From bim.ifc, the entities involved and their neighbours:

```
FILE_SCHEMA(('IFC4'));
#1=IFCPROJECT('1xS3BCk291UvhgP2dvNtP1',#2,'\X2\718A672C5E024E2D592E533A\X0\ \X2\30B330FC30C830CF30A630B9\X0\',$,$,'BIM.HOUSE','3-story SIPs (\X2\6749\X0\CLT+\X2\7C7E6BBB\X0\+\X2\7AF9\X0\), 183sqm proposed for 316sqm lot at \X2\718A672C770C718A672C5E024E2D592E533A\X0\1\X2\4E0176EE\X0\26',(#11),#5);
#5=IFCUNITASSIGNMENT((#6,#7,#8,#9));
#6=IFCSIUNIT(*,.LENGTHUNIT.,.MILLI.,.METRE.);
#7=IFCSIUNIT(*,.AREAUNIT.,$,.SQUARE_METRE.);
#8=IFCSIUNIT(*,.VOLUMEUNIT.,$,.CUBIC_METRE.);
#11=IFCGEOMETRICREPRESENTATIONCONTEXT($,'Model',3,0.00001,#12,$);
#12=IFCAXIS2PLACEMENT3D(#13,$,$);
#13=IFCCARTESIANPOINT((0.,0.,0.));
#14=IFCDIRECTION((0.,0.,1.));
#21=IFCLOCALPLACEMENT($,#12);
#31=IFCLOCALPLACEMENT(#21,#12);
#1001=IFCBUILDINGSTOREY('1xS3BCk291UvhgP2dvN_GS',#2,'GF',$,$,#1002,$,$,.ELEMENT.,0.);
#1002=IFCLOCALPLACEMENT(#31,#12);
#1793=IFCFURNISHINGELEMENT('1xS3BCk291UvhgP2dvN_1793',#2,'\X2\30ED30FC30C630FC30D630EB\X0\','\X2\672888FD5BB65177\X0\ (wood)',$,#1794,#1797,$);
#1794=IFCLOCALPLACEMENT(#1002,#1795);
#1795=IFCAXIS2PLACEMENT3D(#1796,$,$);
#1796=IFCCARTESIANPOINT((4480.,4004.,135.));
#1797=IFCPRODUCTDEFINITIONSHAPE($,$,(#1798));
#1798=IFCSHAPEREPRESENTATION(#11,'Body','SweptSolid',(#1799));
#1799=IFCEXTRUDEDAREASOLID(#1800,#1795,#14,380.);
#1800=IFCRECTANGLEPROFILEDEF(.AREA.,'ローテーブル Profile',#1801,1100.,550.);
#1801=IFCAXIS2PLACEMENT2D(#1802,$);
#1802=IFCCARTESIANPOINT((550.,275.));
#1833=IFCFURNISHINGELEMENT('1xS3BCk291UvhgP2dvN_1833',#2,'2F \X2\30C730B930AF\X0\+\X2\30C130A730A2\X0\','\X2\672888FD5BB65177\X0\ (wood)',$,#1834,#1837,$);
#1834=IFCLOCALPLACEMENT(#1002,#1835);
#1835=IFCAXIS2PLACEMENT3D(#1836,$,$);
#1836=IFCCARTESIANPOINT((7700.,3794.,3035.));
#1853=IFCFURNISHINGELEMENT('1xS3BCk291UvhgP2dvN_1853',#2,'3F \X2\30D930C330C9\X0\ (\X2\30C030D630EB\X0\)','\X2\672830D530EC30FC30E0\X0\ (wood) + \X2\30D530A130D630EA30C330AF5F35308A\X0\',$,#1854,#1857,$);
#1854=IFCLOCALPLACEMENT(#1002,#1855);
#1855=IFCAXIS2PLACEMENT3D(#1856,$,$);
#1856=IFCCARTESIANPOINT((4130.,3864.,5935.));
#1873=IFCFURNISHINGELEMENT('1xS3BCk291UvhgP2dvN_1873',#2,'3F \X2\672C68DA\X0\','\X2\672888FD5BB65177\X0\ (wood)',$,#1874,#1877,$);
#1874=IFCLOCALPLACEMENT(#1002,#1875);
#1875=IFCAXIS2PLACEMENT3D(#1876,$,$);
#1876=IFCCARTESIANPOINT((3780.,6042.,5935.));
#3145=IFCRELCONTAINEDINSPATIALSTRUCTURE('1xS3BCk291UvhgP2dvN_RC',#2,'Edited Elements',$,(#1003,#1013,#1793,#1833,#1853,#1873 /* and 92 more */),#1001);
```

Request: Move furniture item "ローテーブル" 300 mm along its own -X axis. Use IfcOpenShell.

```python
import ifcopenshell
import ifcopenshell.api.geometry
import ifcopenshell.util.placement
import ifcopenshell.util.unit

model = ifcopenshell.open("bim.ifc")
unit_scale = ifcopenshell.util.unit.calculate_unit_scale(model)

item = model.by_id(1793)
matrix = ifcopenshell.util.placement.get_local_placement(item.ObjectPlacement)
matrix[:3, 3] -= matrix[:3, 0] * 0.3 / unit_scale
ifcopenshell.api.geometry.edit_object_placement(model, product=item, matrix=matrix, is_si=False)

print(ifcopenshell.util.placement.get_local_placement(item.ObjectPlacement).round(3) + 0.0)

model.write("bim_v2.ifc")
```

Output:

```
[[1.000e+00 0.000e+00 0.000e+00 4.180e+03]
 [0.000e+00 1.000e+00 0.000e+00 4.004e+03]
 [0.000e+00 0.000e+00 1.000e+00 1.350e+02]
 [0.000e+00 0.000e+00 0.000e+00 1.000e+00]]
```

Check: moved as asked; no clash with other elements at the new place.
